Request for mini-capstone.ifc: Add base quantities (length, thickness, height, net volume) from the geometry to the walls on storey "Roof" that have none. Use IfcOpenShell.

First a look at what the model holds.

```python
import ifcopenshell
import ifcopenshell.util.element
import ifcopenshell.util.unit

model = ifcopenshell.open("mini-capstone.ifc")
print(model.schema)
for unit_type in ("LENGTHUNIT", "AREAUNIT", "VOLUMEUNIT"):
    print(unit_type, ifcopenshell.util.unit.calculate_unit_scale(model, unit_type))
storey = next(s for s in model.by_type("IfcBuildingStorey") if s.Name == "Roof")
walls = [e for e in ifcopenshell.util.element.get_decomposition(storey) if e.is_a("IfcWall")]
for e in sorted(walls, key=lambda e: e.id()):
    print(e.id(), e.is_a(), e.Name, list(ifcopenshell.util.element.get_psets(e, qtos_only=True)), sep=" | ")
```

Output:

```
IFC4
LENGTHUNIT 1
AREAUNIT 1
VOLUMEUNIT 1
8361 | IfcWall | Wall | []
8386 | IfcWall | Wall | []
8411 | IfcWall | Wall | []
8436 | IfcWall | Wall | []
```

```python
import ifcopenshell
import ifcopenshell.api.pset
import ifcopenshell.geom
import ifcopenshell.util.element
import ifcopenshell.util.shape
import ifcopenshell.util.unit

model = ifcopenshell.open("mini-capstone.ifc")
unit_scale = ifcopenshell.util.unit.calculate_unit_scale(model)
volume_scale = ifcopenshell.util.unit.calculate_unit_scale(model, "VOLUMEUNIT")
settings = ifcopenshell.geom.settings()

storey = next(s for s in model.by_type("IfcBuildingStorey") if s.Name == "Roof")
walls = [e for e in ifcopenshell.util.element.get_decomposition(storey) if e.is_a("IfcWall")]

for e in sorted(walls, key=lambda e: e.id()):
    if ifcopenshell.util.element.get_psets(e, qtos_only=True, should_inherit=False):
        continue
    # Geometry comes back in metres, in the element's own axes.
    shape = ifcopenshell.geom.create_shape(settings, e)
    values = {
        "Length": ifcopenshell.util.shape.get_x(shape.geometry) / unit_scale,
        "Width": ifcopenshell.util.shape.get_y(shape.geometry) / unit_scale,
        "Height": ifcopenshell.util.shape.get_z(shape.geometry) / unit_scale,
        "NetVolume": ifcopenshell.util.shape.get_volume(shape.geometry) / volume_scale,
    }
    qto = ifcopenshell.api.pset.add_qto(model, product=e, name="Qto_WallBaseQuantities")
    ifcopenshell.api.pset.edit_qto(model, qto=qto, properties=values)
    print(e.id(), {k: round(v, 3) for k, v in values.items()})

model.write("mini-capstone_v2.ifc")
```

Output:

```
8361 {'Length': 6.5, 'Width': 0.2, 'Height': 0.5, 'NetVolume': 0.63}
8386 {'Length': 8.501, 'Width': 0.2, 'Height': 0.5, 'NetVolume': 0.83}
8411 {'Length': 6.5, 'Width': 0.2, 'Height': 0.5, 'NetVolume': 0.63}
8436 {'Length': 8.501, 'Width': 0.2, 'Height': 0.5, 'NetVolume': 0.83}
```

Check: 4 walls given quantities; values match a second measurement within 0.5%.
